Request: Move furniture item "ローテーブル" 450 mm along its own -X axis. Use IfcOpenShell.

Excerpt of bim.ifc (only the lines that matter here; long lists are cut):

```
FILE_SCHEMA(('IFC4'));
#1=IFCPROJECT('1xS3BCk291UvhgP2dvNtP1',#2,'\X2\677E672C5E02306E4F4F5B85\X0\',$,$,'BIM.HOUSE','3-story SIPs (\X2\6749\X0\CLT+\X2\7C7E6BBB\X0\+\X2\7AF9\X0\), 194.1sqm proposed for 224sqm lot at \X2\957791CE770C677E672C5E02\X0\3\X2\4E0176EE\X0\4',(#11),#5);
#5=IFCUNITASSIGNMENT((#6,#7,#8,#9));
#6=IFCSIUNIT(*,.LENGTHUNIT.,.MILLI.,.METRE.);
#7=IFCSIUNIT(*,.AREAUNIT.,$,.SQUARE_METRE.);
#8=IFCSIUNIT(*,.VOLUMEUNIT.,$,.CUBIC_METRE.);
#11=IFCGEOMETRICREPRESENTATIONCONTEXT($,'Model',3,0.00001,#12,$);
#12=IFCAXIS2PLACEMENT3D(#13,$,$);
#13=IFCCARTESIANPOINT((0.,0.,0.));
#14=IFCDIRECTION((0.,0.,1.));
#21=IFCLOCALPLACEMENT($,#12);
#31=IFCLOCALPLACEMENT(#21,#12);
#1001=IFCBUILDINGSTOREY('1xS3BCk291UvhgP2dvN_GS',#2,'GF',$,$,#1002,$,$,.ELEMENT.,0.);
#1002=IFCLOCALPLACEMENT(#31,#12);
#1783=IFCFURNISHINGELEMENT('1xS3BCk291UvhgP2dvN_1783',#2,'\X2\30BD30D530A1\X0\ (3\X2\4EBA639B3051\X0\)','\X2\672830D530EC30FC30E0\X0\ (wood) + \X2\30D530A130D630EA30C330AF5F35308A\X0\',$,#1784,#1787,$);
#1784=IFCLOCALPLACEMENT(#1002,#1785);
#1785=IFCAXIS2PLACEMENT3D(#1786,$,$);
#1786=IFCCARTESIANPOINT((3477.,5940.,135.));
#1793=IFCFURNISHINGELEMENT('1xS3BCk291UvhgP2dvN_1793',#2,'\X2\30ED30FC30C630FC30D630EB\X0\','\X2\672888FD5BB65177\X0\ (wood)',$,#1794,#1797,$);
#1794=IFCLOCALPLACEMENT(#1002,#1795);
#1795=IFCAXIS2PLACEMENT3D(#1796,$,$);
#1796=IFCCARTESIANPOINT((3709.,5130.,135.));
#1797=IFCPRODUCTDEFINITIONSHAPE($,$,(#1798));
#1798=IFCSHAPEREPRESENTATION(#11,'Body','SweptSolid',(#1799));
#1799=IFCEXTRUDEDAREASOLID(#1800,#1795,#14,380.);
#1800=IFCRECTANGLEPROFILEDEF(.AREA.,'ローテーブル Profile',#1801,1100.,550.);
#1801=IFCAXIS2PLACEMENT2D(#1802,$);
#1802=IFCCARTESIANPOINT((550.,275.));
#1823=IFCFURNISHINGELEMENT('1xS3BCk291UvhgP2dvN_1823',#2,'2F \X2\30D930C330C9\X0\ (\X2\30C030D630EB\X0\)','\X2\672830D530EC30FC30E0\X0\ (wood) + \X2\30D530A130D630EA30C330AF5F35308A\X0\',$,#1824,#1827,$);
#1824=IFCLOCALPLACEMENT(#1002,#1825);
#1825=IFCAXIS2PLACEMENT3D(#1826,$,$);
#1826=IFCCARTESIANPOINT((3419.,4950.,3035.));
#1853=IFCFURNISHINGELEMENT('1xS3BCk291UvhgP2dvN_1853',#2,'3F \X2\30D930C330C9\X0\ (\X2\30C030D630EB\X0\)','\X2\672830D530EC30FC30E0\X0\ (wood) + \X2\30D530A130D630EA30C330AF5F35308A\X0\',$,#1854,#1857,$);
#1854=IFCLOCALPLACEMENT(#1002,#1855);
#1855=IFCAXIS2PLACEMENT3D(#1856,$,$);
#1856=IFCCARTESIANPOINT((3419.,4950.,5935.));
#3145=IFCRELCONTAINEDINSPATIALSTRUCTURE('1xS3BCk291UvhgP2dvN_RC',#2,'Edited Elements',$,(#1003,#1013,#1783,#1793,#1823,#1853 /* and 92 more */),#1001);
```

```python
import ifcopenshell
import ifcopenshell.api.geometry
import ifcopenshell.util.placement

model = ifcopenshell.open("bim.ifc")

item = model.by_guid("1xS3BCk291UvhgP2dvN_1793")
matrix = ifcopenshell.util.placement.get_local_placement(item.ObjectPlacement)
matrix[:3, 3] -= matrix[:3, 0] * 450.0
ifcopenshell.api.geometry.edit_object_placement(model, product=item, matrix=matrix, is_si=False)

print(ifcopenshell.util.placement.get_local_placement(item.ObjectPlacement).round(3) + 0.0)

model.write("bim-out.ifc")
```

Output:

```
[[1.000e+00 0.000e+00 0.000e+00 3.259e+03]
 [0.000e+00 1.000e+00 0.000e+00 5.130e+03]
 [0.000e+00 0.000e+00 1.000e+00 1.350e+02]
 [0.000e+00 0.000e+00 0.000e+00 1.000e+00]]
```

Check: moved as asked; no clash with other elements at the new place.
